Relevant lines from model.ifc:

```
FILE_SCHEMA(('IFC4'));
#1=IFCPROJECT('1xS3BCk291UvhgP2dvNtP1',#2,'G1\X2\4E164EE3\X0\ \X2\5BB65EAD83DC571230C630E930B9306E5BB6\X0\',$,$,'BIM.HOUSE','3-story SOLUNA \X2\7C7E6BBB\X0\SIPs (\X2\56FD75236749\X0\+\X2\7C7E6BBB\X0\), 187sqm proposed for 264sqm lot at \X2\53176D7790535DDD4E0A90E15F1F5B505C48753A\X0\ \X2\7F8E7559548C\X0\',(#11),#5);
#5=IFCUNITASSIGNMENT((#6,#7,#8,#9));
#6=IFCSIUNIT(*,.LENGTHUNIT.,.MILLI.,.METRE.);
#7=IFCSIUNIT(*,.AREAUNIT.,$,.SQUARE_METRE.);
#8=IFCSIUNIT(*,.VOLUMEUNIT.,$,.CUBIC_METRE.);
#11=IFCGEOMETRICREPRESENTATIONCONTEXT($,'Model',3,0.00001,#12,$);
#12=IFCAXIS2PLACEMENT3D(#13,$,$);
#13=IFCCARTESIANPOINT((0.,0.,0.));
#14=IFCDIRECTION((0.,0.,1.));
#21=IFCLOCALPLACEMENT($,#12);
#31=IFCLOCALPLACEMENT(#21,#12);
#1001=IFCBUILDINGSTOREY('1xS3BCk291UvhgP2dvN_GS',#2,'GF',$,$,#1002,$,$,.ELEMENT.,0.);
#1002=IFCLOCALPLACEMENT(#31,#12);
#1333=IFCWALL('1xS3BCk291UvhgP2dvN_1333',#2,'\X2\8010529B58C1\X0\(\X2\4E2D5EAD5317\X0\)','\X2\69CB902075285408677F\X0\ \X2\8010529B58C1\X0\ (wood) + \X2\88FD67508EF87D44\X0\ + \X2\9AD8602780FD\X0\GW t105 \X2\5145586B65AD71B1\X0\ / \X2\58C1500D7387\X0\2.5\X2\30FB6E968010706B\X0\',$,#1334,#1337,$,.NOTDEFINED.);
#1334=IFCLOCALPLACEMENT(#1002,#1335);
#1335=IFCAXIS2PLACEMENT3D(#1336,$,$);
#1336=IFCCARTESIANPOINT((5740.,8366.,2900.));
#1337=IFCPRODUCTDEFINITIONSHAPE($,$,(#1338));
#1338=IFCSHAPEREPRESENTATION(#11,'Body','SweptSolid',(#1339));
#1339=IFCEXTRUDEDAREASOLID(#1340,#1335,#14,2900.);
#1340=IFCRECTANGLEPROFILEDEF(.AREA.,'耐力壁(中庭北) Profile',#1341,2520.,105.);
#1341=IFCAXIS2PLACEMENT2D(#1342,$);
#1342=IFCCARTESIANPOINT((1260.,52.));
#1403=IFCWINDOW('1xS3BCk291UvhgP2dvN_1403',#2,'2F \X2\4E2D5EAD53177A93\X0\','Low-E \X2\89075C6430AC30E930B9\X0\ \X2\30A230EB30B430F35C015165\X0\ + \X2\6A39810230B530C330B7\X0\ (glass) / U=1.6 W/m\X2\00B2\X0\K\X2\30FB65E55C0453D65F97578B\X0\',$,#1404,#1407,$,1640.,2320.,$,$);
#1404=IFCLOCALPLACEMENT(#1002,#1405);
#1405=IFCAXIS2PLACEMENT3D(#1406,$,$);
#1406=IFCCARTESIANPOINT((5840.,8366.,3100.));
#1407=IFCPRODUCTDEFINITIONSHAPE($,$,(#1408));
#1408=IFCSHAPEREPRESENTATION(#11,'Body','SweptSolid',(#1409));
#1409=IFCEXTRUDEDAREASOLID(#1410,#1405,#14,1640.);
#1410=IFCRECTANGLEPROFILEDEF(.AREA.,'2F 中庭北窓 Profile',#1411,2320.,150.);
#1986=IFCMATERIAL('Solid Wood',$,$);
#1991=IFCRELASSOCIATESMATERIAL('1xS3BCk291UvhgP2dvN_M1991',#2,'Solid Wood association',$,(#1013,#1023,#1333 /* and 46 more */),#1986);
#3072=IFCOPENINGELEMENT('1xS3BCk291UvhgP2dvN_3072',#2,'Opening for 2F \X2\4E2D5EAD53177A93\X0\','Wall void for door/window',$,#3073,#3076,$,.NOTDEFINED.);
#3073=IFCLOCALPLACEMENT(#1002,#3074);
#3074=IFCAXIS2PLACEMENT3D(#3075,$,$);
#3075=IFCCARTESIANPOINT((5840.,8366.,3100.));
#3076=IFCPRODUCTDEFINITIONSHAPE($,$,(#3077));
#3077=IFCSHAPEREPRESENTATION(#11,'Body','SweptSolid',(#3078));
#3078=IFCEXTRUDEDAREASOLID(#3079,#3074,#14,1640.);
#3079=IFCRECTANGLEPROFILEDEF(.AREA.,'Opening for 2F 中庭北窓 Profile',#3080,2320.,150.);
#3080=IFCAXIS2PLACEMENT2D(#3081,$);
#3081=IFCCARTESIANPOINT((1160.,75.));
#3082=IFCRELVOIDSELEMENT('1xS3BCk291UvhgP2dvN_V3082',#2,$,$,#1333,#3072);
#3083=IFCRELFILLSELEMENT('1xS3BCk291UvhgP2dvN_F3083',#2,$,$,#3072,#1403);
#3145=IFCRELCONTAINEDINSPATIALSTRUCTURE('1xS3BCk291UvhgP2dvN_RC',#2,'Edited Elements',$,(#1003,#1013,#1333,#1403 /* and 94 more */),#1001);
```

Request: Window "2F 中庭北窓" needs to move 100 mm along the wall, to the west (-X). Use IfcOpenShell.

```python
import ifcopenshell
import ifcopenshell.api.geometry
import ifcopenshell.util.placement
import ifcopenshell.util.unit

model = ifcopenshell.open("model.ifc")
unit_scale = ifcopenshell.util.unit.calculate_unit_scale(model)

window = model.by_id(1403)
opening = window.FillsVoids[0].RelatingOpeningElement
wall = opening.VoidsElements[0].RelatingBuildingElement

wall_matrix = ifcopenshell.util.placement.get_local_placement(wall.ObjectPlacement)
shift = wall_matrix[:3, 0] * -0.1 / unit_scale
before = ifcopenshell.util.placement.get_local_placement(window.ObjectPlacement)[:3, 3].copy()

# The window is not placed relative to its opening, so move both.
for product in (opening, window):
    matrix = ifcopenshell.util.placement.get_local_placement(product.ObjectPlacement)
    matrix[:3, 3] += shift
    ifcopenshell.api.geometry.edit_object_placement(model, product=product, matrix=matrix, is_si=False)

after = ifcopenshell.util.placement.get_local_placement(window.ObjectPlacement)[:3, 3]
print("window moved by", (after - before).round(3) + 0.0)

model.write("model_edited.ifc")
```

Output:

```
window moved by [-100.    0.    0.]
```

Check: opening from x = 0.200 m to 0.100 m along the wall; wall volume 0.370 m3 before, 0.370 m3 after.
